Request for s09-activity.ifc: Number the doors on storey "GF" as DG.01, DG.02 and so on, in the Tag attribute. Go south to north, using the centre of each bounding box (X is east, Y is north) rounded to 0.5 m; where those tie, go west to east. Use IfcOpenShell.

First a look at what the model holds.

```python
import ifcopenshell
import ifcopenshell.util.element
import ifcopenshell.util.placement

model = ifcopenshell.open("s09-activity.ifc")
print(model.schema)
storey = next(s for s in model.by_type("IfcBuildingStorey") if s.Name == "GF")
doors = [e for e in ifcopenshell.util.element.get_decomposition(storey) if e.is_a("IfcDoor")]
for e in sorted(doors, key=lambda e: e.id()):
    origin = ifcopenshell.util.placement.get_local_placement(e.ObjectPlacement)[:3, 3]
    print(e.id(), e.Tag, e.Name, origin.round(2) + 0.0, sep=" | ")
```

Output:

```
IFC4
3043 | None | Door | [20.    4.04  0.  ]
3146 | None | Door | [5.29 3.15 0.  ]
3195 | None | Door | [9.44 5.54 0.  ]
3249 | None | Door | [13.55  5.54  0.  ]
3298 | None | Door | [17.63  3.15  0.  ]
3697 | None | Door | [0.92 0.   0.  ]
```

```python
import ifcopenshell
import ifcopenshell.geom
import ifcopenshell.util.element
import ifcopenshell.util.shape

model = ifcopenshell.open("s09-activity.ifc")
settings = ifcopenshell.geom.settings()
settings.set("use-world-coords", True)


def centre(element):
    shape = ifcopenshell.geom.create_shape(settings, element)
    return ifcopenshell.util.shape.get_bbox_centroid(shape.geometry)


storey = next(s for s in model.by_type("IfcBuildingStorey") if s.Name == "GF")
doors = [e for e in ifcopenshell.util.element.get_decomposition(storey) if e.is_a("IfcDoor")]

# Insertion points can sit at a corner or the storey origin, so sort by the geometry (in metres).
centres = {e: centre(e) for e in doors}
doors.sort(key=lambda e: (round(centres[e][1] / 0.5), centres[e][0]))

for i, e in enumerate(doors, start=1):
    number = f"DG.{i:02d}"
    e.Tag = number
    print(e.id(), number)

model.write("s09-activity_edited.ifc")
```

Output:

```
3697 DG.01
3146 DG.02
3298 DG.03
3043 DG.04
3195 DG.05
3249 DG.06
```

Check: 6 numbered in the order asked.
